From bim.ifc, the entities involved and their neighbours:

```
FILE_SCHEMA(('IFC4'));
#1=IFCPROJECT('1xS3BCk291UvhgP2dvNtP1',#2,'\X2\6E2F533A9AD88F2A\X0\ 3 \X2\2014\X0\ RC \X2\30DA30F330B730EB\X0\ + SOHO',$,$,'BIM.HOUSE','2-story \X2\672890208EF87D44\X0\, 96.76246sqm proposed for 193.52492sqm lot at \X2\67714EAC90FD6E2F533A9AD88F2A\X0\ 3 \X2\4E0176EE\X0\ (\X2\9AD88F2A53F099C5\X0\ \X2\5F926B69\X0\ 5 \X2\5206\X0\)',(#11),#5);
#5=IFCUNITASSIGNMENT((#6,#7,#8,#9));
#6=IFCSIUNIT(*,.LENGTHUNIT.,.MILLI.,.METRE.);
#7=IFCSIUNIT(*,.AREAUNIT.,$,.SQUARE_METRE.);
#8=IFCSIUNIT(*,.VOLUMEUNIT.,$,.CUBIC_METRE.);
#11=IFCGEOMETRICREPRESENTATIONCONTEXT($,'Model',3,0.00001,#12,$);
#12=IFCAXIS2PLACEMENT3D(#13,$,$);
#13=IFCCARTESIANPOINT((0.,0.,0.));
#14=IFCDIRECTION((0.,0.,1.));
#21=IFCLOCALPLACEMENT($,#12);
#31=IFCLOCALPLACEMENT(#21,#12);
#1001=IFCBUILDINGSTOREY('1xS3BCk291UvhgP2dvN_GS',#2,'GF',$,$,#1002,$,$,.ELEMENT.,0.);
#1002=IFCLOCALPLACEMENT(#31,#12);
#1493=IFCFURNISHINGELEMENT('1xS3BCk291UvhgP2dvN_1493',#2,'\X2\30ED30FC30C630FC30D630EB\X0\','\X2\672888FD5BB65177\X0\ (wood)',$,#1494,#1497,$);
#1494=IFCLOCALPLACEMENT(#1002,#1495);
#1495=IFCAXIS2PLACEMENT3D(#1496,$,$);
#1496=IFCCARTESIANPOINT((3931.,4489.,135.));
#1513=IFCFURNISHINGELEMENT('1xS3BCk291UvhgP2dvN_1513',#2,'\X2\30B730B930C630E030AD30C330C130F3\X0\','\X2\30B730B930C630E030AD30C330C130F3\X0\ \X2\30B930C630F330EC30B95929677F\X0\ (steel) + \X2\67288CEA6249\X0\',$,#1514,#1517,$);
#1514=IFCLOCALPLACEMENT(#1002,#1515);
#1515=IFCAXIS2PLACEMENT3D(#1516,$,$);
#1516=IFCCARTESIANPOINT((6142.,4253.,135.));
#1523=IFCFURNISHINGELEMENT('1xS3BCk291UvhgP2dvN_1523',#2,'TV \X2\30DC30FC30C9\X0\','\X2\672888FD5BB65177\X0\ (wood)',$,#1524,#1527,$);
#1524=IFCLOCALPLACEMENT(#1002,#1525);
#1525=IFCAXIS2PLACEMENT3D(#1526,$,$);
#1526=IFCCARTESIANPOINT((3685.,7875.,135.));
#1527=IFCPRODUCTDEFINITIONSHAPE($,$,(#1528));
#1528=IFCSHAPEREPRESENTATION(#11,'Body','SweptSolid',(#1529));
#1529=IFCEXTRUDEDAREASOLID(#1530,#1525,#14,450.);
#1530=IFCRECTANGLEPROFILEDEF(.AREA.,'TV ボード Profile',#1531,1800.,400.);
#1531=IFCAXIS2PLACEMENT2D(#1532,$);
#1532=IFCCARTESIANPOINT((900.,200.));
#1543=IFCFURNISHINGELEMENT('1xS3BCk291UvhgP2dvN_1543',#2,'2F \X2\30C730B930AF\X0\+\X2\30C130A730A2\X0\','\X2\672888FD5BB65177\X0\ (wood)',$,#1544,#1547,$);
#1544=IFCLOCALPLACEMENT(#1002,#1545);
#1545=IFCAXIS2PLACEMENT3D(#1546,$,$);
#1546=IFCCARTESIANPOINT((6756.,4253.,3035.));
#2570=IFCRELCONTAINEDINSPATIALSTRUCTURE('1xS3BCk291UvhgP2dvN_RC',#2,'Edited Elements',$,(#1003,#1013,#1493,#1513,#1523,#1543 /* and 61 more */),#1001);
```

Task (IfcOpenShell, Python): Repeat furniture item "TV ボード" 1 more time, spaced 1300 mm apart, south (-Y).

```python
import numpy as np
import ifcopenshell
import ifcopenshell.api.geometry
import ifcopenshell.api.root
import ifcopenshell.util.element
import ifcopenshell.util.placement

model = ifcopenshell.open("bim.ifc")


def reuse_history(source, copy):
    """copy_class also copies each property set's owner history, people and application; keep the originals."""
    for rel in copy.IsDefinedBy:
        if rel.is_a("IfcRelDefinesByProperties") and (history := rel.RelatingPropertyDefinition.OwnerHistory):
            rel.RelatingPropertyDefinition.OwnerHistory = source.OwnerHistory
            ifcopenshell.util.element.remove_deep2(model, history)


source = model.by_id(1523)
base = ifcopenshell.util.placement.get_local_placement(source.ObjectPlacement)
step = np.array([0.0, -1.0, 0.0]) * 1300.0

for i in range(1, 2):
    copy = ifcopenshell.api.root.copy_class(model, product=source)
    copy.Representation = ifcopenshell.util.element.copy_deep(
        model, source.Representation, exclude=["IfcGeometricRepresentationContext", "IfcRepresentationMap"]
    )
    reuse_history(source, copy)
    matrix = base.copy()
    matrix[:3, 3] += i * step
    print("added at", matrix[:3, 3].round(3) + 0.0)
    ifcopenshell.api.geometry.edit_object_placement(model, product=copy, matrix=matrix, is_si=False)

model.write("bim_updated.ifc")
```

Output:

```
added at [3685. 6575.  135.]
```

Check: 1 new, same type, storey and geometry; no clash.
